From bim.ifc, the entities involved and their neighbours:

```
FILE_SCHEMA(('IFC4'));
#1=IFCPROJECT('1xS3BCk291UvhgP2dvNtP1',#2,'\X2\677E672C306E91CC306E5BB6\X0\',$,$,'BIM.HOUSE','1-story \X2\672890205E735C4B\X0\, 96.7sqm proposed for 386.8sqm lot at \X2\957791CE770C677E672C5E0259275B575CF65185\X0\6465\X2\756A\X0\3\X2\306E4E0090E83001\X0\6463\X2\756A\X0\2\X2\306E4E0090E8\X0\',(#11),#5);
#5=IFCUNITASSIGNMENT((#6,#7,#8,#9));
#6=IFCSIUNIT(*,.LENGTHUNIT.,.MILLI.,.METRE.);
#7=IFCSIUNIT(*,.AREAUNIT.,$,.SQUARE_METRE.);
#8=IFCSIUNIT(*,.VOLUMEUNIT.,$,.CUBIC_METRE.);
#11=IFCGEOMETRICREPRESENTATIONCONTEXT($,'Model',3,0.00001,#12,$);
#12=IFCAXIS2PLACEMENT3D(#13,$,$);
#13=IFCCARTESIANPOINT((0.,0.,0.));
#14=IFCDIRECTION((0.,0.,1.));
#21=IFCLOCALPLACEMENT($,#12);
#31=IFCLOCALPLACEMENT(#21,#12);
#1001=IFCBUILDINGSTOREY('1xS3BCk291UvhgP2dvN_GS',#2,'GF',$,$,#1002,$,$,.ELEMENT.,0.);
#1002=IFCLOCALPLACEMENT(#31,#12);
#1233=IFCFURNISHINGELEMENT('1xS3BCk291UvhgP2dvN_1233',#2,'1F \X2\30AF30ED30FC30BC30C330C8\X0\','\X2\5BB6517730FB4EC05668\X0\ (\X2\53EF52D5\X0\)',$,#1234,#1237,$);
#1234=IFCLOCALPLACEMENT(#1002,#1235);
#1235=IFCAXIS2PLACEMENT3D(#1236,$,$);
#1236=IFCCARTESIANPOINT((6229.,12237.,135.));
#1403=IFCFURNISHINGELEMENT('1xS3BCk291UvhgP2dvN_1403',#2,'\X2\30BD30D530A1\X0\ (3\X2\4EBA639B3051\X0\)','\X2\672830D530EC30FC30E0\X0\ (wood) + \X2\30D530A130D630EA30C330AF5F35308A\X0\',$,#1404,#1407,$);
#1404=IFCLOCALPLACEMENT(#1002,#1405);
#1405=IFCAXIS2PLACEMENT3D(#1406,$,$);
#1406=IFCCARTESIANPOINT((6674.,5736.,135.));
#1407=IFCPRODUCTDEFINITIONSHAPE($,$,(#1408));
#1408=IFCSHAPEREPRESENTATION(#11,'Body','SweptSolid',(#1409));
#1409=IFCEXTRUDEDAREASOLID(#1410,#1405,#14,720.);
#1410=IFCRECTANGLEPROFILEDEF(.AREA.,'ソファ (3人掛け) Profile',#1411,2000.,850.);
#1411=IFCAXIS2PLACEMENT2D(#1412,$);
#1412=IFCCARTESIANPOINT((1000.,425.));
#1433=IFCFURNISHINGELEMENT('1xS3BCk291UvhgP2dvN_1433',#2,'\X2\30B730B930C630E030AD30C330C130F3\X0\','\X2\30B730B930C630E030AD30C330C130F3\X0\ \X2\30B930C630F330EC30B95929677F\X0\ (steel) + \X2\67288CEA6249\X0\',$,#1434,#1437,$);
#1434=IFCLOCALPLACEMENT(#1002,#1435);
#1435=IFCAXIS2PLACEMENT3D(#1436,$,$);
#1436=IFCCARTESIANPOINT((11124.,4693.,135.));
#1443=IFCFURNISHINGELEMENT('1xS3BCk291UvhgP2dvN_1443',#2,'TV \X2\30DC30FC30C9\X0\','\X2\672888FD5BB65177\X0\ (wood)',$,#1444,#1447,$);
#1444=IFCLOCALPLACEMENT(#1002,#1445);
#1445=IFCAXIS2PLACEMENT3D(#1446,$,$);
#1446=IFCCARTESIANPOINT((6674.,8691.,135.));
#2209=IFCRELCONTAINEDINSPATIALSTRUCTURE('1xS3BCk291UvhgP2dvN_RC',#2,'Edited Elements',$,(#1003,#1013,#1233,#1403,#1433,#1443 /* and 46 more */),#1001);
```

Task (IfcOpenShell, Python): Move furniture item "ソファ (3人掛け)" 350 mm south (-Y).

```python
import ifcopenshell
import ifcopenshell.api.geometry
import ifcopenshell.util.placement

model = ifcopenshell.open("bim.ifc")

item = model.by_guid("1xS3BCk291UvhgP2dvN_1403")
matrix = ifcopenshell.util.placement.get_local_placement(item.ObjectPlacement)
matrix[1, 3] -= 350.0
ifcopenshell.api.geometry.edit_object_placement(model, product=item, matrix=matrix, is_si=False)

print(ifcopenshell.util.placement.get_local_placement(item.ObjectPlacement).round(3) + 0.0)

model.write("bim-out.ifc")
```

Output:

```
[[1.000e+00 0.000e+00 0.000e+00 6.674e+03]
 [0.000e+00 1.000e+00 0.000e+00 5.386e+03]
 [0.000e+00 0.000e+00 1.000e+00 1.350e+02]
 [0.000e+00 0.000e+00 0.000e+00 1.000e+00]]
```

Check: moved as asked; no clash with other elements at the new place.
